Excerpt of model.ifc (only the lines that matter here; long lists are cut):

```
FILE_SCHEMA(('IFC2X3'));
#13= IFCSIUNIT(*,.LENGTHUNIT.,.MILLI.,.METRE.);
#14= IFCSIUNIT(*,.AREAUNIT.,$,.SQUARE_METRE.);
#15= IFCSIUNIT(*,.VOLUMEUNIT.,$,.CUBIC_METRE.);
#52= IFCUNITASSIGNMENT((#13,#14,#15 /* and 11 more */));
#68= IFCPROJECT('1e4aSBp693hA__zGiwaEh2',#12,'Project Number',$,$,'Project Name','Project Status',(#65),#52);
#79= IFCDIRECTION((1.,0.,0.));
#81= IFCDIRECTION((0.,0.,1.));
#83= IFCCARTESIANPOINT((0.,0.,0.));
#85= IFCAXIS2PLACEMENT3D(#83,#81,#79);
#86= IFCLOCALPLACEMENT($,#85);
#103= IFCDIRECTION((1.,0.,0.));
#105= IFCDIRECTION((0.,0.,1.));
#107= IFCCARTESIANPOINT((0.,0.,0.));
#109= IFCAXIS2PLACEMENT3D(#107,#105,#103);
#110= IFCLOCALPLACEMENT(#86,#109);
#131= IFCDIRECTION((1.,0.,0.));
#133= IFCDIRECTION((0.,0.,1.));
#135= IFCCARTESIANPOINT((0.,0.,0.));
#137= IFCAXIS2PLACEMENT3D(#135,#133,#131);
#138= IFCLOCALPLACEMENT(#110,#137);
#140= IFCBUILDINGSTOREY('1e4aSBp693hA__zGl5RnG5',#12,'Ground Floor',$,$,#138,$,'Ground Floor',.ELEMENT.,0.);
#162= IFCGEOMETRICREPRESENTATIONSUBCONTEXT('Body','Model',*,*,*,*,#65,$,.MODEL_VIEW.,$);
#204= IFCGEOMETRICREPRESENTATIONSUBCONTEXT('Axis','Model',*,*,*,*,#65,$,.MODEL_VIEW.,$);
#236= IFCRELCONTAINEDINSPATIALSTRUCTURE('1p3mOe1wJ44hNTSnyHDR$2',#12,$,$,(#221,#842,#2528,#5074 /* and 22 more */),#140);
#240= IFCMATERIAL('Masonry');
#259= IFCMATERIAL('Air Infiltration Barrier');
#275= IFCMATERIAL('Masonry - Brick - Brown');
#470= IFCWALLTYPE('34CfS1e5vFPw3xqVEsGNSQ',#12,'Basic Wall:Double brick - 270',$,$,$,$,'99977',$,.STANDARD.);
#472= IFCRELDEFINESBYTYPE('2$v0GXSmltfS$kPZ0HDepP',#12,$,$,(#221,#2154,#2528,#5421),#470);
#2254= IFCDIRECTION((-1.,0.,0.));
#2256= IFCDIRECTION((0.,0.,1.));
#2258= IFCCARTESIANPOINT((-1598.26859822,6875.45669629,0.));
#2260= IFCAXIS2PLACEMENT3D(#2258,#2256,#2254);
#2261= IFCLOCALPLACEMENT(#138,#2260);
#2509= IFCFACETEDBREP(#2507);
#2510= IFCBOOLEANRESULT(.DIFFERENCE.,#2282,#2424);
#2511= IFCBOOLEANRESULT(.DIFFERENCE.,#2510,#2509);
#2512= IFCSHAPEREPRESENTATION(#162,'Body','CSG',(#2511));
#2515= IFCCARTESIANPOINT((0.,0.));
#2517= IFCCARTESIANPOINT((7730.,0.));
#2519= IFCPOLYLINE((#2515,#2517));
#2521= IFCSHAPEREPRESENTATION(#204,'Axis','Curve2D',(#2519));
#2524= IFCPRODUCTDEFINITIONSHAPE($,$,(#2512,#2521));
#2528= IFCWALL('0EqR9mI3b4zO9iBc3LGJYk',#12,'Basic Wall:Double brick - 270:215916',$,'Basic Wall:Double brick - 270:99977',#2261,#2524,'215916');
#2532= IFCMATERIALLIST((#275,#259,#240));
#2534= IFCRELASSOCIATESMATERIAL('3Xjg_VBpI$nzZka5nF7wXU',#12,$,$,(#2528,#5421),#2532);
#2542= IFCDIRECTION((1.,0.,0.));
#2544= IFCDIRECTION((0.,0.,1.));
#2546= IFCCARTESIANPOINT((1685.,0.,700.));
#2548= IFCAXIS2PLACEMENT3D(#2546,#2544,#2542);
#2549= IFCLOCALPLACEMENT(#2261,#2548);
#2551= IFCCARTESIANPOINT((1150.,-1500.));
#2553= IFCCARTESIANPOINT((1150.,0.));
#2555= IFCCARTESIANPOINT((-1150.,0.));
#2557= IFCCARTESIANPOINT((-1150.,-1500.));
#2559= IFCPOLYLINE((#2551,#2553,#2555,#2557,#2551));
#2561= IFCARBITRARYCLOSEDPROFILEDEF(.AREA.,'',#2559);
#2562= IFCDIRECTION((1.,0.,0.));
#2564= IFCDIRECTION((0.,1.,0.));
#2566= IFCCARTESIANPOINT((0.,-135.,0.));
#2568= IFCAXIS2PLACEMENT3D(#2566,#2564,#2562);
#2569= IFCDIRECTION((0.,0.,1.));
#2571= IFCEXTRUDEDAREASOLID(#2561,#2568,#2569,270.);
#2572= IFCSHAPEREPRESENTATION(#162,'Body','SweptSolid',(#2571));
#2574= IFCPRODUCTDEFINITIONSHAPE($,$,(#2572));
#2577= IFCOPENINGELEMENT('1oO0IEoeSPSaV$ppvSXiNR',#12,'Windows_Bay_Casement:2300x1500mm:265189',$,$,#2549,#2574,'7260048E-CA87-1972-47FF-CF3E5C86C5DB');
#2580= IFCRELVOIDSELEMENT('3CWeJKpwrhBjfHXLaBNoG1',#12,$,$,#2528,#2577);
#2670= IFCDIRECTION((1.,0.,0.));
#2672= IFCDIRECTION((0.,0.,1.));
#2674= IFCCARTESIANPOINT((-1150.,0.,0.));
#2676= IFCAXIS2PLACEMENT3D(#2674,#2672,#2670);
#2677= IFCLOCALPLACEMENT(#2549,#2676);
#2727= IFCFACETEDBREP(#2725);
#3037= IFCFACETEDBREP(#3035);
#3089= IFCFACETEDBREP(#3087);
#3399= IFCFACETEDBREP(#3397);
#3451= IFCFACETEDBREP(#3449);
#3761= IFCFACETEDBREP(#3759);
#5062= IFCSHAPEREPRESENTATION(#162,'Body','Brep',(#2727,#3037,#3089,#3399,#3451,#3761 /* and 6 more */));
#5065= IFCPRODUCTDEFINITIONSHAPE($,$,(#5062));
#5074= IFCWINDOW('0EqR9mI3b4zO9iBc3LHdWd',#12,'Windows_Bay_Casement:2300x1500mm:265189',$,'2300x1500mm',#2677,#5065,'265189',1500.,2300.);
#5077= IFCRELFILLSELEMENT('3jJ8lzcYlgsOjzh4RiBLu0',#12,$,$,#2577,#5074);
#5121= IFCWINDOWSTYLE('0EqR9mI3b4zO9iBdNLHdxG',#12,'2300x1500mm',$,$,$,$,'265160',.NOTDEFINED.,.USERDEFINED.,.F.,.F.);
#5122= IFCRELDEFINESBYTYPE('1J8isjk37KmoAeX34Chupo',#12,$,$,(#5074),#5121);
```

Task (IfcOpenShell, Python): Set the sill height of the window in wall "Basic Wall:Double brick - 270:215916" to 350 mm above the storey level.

```python
import numpy as np
import ifcopenshell
import ifcopenshell.api.geometry
import ifcopenshell.geom
import ifcopenshell.util.element
import ifcopenshell.util.placement
import ifcopenshell.util.shape
import ifcopenshell.util.unit

model = ifcopenshell.open("model.ifc")
unit_scale = ifcopenshell.util.unit.calculate_unit_scale(model)

window = model.by_guid("0EqR9mI3b4zO9iBc3LHdWd")
opening = window.FillsVoids[0].RelatingOpeningElement
storey = ifcopenshell.util.element.get_container(window, ifc_class="IfcBuildingStorey")
level = ifcopenshell.util.placement.get_local_placement(storey.ObjectPlacement)[2, 3]

# The opening's origin need not be at the sill, so measure its lowest point.
shape = ifcopenshell.geom.create_shape(ifcopenshell.geom.settings(), opening)
bottom = ifcopenshell.util.shape.get_shape_bottom_elevation(shape, shape.geometry) / unit_scale
dz = level + 0.35 / unit_scale - bottom

shift = np.array([0.0, 0.0, dz])
# The window is placed relative to its opening, so it follows when the opening moves.
matrix = ifcopenshell.util.placement.get_local_placement(opening.ObjectPlacement)
matrix[:3, 3] += shift
ifcopenshell.api.geometry.edit_object_placement(
    model, product=opening, matrix=matrix, is_si=False, should_transform_children=True
)

print(f"moved by {dz * unit_scale:+.3f} m")

model.write("model_v2.ifc")
```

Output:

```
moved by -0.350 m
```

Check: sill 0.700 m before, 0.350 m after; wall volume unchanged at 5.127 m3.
